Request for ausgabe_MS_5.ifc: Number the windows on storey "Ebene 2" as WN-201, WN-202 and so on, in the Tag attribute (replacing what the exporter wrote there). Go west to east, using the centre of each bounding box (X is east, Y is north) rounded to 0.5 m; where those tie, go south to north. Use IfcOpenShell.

First a look at what the model holds.

```python
import ifcopenshell
import ifcopenshell.util.element
import ifcopenshell.util.placement

model = ifcopenshell.open("ausgabe_MS_5.ifc")
print(model.schema)
storey = next(s for s in model.by_type("IfcBuildingStorey") if s.Name == "Ebene 2")
windows = [e for e in ifcopenshell.util.element.get_decomposition(storey) if e.is_a("IfcWindow")]
for e in sorted(windows, key=lambda e: e.id()):
    origin = ifcopenshell.util.placement.get_local_placement(e.ObjectPlacement)[:3, 3]
    print(e.id(), e.Tag, e.Name, origin.round(2) + 0.0, sep=" | ")
```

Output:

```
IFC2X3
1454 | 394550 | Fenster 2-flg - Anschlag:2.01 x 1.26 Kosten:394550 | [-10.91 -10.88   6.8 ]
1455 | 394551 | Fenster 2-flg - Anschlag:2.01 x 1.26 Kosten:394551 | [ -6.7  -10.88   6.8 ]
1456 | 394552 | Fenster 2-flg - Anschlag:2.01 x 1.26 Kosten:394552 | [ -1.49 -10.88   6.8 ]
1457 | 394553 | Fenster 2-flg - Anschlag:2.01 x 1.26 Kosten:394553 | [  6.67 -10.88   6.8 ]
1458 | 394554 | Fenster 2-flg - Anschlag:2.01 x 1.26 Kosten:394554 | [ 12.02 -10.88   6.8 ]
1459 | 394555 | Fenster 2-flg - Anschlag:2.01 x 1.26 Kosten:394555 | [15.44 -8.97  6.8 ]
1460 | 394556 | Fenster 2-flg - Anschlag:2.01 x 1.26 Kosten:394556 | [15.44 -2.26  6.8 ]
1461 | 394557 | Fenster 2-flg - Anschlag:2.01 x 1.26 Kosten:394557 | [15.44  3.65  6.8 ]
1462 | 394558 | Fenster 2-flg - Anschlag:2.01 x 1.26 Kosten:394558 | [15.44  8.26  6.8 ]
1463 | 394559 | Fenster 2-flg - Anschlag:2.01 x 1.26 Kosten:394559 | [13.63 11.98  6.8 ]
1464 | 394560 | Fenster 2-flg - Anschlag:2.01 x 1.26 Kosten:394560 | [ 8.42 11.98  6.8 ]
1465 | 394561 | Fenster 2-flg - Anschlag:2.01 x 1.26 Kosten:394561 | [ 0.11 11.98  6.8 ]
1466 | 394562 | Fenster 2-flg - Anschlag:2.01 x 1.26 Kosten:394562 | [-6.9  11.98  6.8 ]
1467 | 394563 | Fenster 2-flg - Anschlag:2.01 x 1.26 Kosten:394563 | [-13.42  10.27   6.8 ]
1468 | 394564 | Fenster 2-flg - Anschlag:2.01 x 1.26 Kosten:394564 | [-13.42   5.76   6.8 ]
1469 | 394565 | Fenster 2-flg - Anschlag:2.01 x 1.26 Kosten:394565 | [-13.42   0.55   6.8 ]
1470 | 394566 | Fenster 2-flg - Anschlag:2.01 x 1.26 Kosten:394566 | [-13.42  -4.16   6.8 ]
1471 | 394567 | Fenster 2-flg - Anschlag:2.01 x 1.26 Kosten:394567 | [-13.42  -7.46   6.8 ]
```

```python
import ifcopenshell
import ifcopenshell.geom
import ifcopenshell.util.element
import ifcopenshell.util.shape

model = ifcopenshell.open("ausgabe_MS_5.ifc")
settings = ifcopenshell.geom.settings()
settings.set("use-world-coords", True)


def centre(element):
    shape = ifcopenshell.geom.create_shape(settings, element)
    return ifcopenshell.util.shape.get_bbox_centroid(shape.geometry)


storey = next(s for s in model.by_type("IfcBuildingStorey") if s.Name == "Ebene 2")
windows = [e for e in ifcopenshell.util.element.get_decomposition(storey) if e.is_a("IfcWindow")]

# Insertion points can sit at a corner or the storey origin, so sort by the geometry (in metres).
centres = {e: centre(e) for e in windows}
windows.sort(key=lambda e: (round(centres[e][0] / 0.5), centres[e][1]))

for i, e in enumerate(windows, start=1):
    number = f"WN-2{i:02d}"
    e.Tag = number
    print(e.id(), number)

model.write("ausgabe_MS_5_edited.ifc")
```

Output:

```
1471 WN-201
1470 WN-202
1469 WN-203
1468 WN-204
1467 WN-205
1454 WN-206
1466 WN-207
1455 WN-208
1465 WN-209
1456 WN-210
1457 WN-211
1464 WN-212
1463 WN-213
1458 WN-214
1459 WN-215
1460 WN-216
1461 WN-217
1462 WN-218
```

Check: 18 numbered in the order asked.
